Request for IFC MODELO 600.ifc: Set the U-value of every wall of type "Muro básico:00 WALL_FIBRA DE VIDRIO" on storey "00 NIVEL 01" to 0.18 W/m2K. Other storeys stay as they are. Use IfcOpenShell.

First a look at what the model holds.

```python
import ifcopenshell
import ifcopenshell.util.element

model = ifcopenshell.open("IFC MODELO 600.ifc")
print(model.schema)
storey = next(s for s in model.by_type("IfcBuildingStorey") if s.Name == "00 NIVEL 01")
walls = [e for e in ifcopenshell.util.element.get_decomposition(storey) if e.is_a("IfcWall")]
seen = {}
for e in walls:
    element_type = ifcopenshell.util.element.get_type(e)
    key = (element_type.Name if element_type != e and element_type else None, ifcopenshell.util.element.get_pset(e, "Pset_WallCommon", "ThermalTransmittance"))
    seen[key] = seen.get(key, 0) + 1
for (name, value), count in sorted(seen.items(), key=str):
    print(count, "x", name, "|", value)
```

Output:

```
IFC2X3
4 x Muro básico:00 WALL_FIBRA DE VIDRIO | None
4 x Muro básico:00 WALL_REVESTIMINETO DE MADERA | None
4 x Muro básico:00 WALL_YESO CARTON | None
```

```python
import ifcopenshell
import ifcopenshell.api.pset
import ifcopenshell.util.element

model = ifcopenshell.open("IFC MODELO 600.ifc")

storey = next(s for s in model.by_type("IfcBuildingStorey") if s.Name == "00 NIVEL 01")
walls = [e for e in ifcopenshell.util.element.get_decomposition(storey) if e.is_a("IfcWall")]

count = 0
for e in walls:
    element_type = ifcopenshell.util.element.get_type(e)
    if element_type in (None, e) or element_type.Name != "Muro básico:00 WALL_FIBRA DE VIDRIO":
        continue
    # add_pset returns the element's existing set when there is one.
    pset = ifcopenshell.api.pset.add_pset(model, product=e, name="Pset_WallCommon")
    ifcopenshell.api.pset.edit_pset(model, pset=pset, properties={"ThermalTransmittance": 0.18})
    count += 1

print(count, "walls updated")

model.write("IFC MODELO 600_updated.ifc")
```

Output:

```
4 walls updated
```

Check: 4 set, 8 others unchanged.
